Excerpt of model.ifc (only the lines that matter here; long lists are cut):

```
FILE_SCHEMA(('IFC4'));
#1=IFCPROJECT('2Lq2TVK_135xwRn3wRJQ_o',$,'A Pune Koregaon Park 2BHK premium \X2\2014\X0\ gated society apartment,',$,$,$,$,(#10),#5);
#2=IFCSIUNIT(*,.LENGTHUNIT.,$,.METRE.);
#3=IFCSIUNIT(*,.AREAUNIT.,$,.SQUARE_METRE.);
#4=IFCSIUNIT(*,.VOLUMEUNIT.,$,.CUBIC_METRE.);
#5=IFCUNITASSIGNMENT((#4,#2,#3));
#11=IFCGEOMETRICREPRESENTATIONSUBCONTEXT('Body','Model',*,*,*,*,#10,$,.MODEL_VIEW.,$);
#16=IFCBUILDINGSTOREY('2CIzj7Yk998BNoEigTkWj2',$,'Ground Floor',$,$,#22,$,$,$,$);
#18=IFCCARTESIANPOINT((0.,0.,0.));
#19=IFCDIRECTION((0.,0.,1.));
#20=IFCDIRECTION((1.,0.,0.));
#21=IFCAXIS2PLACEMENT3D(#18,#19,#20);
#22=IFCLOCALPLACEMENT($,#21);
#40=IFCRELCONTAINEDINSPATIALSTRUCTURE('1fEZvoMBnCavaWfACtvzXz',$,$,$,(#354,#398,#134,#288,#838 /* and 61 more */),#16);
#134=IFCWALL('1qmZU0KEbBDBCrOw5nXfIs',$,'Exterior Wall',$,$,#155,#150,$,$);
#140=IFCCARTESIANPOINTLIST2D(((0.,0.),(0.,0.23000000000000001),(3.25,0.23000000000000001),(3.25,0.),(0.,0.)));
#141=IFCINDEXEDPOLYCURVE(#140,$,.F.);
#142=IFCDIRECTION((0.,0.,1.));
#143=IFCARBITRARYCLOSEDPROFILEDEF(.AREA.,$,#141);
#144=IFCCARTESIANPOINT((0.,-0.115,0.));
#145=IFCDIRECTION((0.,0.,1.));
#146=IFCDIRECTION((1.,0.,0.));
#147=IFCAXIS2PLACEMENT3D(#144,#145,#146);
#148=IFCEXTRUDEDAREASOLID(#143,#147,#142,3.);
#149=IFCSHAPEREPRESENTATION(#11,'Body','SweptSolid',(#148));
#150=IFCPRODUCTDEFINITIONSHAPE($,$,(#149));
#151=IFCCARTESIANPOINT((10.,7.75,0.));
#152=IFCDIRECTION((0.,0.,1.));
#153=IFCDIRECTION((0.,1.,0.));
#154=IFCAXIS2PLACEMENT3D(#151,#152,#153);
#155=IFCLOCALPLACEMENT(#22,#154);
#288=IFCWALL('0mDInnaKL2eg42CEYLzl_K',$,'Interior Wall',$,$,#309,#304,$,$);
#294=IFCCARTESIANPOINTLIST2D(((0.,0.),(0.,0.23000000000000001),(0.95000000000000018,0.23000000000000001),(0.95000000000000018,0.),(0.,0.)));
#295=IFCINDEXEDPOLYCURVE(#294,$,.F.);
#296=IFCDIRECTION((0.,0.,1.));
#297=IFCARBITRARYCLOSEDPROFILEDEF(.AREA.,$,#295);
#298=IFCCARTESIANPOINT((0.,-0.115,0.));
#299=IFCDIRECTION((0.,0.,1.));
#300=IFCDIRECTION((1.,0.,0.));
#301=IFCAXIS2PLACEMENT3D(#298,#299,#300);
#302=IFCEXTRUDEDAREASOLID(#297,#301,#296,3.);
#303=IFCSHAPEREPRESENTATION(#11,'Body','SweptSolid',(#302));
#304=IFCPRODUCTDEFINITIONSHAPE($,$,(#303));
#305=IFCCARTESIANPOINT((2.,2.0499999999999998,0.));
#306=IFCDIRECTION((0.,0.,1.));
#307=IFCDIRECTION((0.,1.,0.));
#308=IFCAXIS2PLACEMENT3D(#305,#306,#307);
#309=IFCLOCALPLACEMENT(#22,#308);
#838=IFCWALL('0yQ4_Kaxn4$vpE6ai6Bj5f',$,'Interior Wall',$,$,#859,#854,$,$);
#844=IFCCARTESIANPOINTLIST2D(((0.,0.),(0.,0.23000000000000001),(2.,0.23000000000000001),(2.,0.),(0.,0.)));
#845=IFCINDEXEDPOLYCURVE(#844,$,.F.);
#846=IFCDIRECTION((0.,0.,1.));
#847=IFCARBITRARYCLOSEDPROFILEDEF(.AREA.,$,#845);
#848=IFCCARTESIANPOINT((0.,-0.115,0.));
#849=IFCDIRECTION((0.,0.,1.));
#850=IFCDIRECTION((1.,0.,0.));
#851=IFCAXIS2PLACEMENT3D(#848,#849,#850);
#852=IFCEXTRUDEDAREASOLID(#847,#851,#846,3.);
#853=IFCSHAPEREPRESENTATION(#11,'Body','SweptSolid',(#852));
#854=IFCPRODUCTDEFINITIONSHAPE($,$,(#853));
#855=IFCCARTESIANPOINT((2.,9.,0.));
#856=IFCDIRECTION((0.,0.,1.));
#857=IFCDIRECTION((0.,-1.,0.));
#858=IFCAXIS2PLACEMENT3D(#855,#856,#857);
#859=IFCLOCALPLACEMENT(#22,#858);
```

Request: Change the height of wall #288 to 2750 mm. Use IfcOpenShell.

```python
import ifcopenshell
import ifcopenshell.geom
import ifcopenshell.util.representation
import ifcopenshell.util.shape
import ifcopenshell.util.unit

model = ifcopenshell.open("model.ifc")
unit_scale = ifcopenshell.util.unit.calculate_unit_scale(model)
settings = ifcopenshell.geom.settings()


def volume(element):
    """Net volume in cubic metres, openings subtracted."""
    shape = ifcopenshell.geom.create_shape(settings, element)
    return ifcopenshell.util.shape.get_volume(shape.geometry)


wall = model.by_guid("0mDInnaKL2eg42CEYLzl_K")
before = volume(wall)

body = ifcopenshell.util.representation.get_representation(wall, "Model", "Body")
solid = body.Items[0]
old_height = solid.Depth
solid.Depth = 2.75 / unit_scale
after = volume(wall)

print(f"height {old_height:g} -> {solid.Depth:g}, volume {before:.3f} -> {after:.3f} m3")

model.write("model_updated.ifc")
```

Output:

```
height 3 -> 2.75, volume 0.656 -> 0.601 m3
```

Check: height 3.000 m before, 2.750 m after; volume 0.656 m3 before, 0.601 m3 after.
